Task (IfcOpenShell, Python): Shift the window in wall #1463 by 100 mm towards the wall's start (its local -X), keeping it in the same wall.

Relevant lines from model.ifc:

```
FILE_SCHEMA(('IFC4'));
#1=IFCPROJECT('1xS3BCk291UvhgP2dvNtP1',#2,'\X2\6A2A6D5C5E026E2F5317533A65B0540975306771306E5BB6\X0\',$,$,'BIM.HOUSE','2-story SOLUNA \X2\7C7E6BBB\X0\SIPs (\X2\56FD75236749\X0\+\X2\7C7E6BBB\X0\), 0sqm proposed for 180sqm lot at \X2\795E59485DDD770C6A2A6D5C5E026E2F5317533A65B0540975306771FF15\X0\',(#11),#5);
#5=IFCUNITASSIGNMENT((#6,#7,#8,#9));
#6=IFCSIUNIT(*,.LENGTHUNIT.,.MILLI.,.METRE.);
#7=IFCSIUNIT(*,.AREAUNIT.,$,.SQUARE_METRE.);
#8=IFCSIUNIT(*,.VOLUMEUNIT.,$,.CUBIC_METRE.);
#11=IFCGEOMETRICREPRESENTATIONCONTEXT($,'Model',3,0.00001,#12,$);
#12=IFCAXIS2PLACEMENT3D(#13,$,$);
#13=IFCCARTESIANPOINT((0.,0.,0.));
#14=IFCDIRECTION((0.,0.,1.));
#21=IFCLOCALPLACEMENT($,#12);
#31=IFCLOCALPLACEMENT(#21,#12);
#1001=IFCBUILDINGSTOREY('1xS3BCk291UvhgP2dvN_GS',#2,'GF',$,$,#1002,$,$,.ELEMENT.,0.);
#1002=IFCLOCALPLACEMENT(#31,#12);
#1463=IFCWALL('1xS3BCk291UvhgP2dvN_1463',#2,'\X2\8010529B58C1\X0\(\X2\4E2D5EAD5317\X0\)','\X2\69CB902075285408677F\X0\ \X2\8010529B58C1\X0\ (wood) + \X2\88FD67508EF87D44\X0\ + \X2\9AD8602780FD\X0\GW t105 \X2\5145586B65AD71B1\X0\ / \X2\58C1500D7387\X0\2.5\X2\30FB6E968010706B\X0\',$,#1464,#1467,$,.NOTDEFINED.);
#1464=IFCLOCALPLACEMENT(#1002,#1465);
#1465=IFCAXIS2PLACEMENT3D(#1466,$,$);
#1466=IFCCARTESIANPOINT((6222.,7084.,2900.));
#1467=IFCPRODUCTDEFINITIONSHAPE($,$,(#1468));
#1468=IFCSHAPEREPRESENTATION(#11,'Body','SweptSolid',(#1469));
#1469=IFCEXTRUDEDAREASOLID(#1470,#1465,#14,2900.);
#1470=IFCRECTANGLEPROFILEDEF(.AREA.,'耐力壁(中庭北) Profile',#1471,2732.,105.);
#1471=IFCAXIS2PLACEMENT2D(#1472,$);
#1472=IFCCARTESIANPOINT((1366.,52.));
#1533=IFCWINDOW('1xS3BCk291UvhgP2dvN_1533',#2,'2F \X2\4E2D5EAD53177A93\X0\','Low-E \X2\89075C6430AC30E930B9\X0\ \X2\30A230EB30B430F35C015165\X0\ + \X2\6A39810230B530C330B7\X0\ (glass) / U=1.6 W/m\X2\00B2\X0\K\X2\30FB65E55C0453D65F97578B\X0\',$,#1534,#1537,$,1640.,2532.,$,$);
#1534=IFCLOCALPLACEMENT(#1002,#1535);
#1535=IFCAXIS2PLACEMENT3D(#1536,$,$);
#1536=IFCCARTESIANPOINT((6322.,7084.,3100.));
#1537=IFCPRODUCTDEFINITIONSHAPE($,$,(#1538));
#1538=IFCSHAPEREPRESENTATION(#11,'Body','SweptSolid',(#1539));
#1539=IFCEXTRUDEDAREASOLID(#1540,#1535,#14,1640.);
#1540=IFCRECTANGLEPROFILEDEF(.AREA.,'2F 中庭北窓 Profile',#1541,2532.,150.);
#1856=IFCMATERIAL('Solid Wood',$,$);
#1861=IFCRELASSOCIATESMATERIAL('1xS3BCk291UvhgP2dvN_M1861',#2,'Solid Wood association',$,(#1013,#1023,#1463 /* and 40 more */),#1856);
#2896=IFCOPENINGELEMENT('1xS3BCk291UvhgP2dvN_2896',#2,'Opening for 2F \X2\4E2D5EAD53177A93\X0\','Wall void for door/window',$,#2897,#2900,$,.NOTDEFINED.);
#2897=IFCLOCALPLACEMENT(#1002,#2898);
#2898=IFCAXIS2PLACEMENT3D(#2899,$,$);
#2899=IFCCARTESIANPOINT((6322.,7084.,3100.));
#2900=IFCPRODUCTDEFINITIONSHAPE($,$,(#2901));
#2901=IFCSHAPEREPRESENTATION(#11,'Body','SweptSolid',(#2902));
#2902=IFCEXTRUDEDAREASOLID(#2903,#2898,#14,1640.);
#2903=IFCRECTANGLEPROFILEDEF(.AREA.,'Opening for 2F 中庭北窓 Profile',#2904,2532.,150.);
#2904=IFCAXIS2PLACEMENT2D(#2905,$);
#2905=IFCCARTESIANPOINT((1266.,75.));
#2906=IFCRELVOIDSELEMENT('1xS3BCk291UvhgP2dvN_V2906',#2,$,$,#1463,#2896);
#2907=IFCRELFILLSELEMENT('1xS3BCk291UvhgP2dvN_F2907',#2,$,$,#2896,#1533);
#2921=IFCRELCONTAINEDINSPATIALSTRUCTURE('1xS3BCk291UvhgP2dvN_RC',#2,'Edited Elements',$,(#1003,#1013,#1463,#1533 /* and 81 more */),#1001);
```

```python
import ifcopenshell
import ifcopenshell.api.geometry
import ifcopenshell.util.placement
import ifcopenshell.util.unit

model = ifcopenshell.open("model.ifc")
unit_scale = ifcopenshell.util.unit.calculate_unit_scale(model)

window = model.by_guid("1xS3BCk291UvhgP2dvN_1533")
opening = window.FillsVoids[0].RelatingOpeningElement
wall = opening.VoidsElements[0].RelatingBuildingElement

wall_matrix = ifcopenshell.util.placement.get_local_placement(wall.ObjectPlacement)
shift = wall_matrix[:3, 0] * -0.1 / unit_scale
before = ifcopenshell.util.placement.get_local_placement(window.ObjectPlacement)[:3, 3].copy()

# The window is not placed relative to its opening, so move both.
for product in (opening, window):
    matrix = ifcopenshell.util.placement.get_local_placement(product.ObjectPlacement)
    matrix[:3, 3] += shift
    ifcopenshell.api.geometry.edit_object_placement(model, product=product, matrix=matrix, is_si=False)

after = ifcopenshell.util.placement.get_local_placement(window.ObjectPlacement)[:3, 3]
print("window moved by", (after - before).round(3) + 0.0)

model.write("model-out.ifc")
```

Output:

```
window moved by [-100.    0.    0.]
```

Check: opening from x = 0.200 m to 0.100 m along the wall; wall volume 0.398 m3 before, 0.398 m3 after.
